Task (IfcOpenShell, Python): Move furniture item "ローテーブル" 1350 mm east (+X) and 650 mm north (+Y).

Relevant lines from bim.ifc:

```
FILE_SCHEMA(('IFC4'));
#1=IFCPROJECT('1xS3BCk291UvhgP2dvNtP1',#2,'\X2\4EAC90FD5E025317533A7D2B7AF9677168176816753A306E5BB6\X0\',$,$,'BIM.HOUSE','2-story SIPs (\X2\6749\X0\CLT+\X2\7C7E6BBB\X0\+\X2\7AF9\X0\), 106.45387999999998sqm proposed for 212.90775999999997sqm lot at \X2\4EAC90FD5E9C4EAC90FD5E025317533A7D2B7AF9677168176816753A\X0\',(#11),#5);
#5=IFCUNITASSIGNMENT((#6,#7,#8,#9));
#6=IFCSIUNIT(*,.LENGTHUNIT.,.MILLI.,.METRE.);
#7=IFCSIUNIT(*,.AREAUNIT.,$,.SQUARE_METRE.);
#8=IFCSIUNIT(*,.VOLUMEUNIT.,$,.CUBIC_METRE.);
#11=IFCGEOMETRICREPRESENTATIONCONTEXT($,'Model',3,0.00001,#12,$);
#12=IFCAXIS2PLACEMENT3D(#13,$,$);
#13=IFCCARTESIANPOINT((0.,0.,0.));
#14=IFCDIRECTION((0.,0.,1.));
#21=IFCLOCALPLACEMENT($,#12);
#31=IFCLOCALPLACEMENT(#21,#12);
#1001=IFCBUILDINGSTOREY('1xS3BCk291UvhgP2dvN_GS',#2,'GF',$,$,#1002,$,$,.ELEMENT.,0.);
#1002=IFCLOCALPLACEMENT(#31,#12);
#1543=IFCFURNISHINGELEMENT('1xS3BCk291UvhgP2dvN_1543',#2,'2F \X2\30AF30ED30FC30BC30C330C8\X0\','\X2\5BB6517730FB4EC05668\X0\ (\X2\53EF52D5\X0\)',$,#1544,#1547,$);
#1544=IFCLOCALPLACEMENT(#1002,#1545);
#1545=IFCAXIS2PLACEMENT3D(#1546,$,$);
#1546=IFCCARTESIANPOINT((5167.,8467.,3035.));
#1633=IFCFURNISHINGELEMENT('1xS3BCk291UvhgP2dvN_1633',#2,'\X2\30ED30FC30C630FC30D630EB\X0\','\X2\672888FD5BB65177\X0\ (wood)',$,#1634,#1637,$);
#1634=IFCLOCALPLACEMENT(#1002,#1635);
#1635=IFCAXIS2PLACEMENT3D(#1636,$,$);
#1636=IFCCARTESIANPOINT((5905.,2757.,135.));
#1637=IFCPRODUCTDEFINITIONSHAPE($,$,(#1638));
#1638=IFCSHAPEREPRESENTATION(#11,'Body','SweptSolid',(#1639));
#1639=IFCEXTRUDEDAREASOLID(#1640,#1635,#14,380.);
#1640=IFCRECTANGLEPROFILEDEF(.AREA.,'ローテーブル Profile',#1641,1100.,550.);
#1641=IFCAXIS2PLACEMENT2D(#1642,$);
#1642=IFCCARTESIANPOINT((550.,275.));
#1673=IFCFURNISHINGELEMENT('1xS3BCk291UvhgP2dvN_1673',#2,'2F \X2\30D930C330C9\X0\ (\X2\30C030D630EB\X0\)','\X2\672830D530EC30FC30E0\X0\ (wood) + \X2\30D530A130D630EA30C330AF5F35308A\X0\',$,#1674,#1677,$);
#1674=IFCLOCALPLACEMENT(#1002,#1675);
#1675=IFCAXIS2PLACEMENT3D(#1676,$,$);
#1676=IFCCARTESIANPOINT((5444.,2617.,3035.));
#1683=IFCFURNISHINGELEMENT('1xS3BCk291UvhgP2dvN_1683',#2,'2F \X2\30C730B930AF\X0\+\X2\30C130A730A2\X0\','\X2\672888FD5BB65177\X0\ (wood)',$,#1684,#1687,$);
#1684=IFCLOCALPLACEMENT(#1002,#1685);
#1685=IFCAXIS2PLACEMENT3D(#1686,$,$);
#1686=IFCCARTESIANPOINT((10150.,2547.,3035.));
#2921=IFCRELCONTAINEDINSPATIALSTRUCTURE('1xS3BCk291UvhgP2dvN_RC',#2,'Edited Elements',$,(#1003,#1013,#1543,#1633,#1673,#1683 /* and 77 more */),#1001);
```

```python
import ifcopenshell
import ifcopenshell.api.geometry
import ifcopenshell.util.placement

model = ifcopenshell.open("bim.ifc")

item = model.by_guid("1xS3BCk291UvhgP2dvN_1633")
matrix = ifcopenshell.util.placement.get_local_placement(item.ObjectPlacement)
matrix[0, 3] += 1350.0
matrix[1, 3] += 650.0
ifcopenshell.api.geometry.edit_object_placement(model, product=item, matrix=matrix, is_si=False)

print(ifcopenshell.util.placement.get_local_placement(item.ObjectPlacement).round(3) + 0.0)

model.write("bim_updated.ifc")
```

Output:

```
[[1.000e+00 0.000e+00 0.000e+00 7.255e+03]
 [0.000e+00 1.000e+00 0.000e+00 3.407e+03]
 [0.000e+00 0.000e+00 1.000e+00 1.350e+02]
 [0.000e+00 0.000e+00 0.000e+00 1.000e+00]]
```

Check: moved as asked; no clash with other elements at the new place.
